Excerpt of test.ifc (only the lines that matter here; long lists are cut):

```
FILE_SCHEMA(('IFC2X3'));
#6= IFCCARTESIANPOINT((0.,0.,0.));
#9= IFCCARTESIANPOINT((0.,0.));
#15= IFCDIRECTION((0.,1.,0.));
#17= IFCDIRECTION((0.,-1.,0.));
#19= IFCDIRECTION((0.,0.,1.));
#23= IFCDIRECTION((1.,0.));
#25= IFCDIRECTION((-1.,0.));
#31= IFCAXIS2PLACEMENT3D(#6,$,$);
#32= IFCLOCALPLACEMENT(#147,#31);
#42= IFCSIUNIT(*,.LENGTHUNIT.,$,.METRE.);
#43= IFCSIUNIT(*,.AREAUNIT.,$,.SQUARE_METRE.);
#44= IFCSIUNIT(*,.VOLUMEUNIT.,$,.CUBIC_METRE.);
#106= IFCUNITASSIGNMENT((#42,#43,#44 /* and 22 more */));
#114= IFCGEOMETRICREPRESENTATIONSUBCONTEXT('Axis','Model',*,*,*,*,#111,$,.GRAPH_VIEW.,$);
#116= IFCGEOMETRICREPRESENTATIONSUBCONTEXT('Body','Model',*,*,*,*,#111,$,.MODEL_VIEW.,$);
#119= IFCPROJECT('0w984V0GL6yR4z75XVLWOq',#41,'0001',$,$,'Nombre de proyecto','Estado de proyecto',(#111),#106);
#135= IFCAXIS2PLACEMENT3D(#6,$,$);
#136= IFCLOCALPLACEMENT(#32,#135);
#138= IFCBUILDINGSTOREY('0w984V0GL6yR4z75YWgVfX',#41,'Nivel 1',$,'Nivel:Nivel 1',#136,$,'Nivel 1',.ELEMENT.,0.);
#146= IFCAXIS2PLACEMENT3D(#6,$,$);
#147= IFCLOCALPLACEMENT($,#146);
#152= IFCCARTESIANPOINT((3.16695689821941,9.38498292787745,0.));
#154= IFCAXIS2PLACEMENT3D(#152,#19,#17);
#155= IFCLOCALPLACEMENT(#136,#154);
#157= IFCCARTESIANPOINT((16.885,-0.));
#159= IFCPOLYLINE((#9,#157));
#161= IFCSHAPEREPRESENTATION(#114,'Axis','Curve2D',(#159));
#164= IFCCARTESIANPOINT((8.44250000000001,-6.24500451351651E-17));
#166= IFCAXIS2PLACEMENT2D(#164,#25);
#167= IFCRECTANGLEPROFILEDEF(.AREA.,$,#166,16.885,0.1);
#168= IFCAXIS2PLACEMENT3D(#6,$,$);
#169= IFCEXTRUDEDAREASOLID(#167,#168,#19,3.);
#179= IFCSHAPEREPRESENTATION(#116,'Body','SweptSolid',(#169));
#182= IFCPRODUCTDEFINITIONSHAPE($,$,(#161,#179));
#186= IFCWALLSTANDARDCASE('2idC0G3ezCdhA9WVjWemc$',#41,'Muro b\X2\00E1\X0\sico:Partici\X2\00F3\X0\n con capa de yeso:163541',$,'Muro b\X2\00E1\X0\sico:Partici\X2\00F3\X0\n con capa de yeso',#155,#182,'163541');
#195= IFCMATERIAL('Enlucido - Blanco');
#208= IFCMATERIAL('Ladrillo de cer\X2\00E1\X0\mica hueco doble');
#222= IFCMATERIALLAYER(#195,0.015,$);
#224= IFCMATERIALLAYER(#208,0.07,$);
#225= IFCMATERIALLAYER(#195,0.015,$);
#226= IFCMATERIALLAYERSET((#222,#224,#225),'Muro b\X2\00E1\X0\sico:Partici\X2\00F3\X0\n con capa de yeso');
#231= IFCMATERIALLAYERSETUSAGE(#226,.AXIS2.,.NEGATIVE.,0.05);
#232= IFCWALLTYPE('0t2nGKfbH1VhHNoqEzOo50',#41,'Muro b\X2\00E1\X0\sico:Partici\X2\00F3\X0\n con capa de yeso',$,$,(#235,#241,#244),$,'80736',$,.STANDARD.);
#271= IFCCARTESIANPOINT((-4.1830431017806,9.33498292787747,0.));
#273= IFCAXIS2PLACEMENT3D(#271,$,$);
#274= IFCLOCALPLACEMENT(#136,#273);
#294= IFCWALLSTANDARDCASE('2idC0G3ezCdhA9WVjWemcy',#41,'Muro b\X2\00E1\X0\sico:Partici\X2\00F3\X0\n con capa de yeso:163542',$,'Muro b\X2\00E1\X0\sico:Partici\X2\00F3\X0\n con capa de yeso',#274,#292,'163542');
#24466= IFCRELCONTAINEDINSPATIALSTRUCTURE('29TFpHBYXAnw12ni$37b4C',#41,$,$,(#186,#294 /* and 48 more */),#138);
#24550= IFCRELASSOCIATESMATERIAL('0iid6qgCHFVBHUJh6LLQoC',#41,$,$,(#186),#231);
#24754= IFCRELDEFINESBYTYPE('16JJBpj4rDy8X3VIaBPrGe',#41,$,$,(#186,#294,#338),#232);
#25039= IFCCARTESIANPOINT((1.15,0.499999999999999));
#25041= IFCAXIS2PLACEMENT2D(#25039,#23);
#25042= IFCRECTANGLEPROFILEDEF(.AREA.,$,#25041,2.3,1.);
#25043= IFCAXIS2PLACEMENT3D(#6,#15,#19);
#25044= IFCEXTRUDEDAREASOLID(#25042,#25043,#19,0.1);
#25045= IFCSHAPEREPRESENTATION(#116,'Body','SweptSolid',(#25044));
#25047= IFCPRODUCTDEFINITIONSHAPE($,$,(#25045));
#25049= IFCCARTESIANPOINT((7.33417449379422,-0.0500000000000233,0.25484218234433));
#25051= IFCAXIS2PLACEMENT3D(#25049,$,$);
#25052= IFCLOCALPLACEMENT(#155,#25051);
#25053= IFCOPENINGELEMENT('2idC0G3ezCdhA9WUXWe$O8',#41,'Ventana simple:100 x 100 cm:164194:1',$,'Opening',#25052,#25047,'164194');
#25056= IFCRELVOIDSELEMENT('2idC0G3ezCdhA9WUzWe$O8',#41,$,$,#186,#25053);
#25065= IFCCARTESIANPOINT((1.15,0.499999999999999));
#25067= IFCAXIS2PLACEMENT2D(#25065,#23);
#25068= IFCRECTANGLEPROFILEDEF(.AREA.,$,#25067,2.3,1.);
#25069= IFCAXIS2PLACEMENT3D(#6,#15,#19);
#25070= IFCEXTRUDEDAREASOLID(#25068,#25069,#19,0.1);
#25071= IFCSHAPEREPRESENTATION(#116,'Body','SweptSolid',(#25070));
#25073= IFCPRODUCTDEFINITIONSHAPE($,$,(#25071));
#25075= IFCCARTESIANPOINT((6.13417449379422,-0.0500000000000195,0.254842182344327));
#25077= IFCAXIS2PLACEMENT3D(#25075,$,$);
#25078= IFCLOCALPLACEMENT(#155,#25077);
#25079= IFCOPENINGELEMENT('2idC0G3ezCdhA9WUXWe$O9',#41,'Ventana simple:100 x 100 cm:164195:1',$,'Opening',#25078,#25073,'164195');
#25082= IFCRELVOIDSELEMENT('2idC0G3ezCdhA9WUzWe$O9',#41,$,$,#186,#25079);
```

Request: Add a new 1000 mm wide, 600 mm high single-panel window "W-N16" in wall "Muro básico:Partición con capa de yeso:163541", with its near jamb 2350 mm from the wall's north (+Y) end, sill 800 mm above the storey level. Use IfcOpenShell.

```python
import numpy as np
import ifcopenshell
import ifcopenshell.api.feature
import ifcopenshell.api.geometry
import ifcopenshell.api.root
import ifcopenshell.api.spatial
import ifcopenshell.api.type
import ifcopenshell.geom
import ifcopenshell.util.element
import ifcopenshell.util.placement
import ifcopenshell.util.representation
import ifcopenshell.util.shape
import ifcopenshell.util.unit

model = ifcopenshell.open("test.ifc")
unit_scale = ifcopenshell.util.unit.calculate_unit_scale(model)
settings = ifcopenshell.geom.settings()


def volume(element):
    """Net volume in cubic metres, openings subtracted."""
    shape = ifcopenshell.geom.create_shape(settings, element)
    return ifcopenshell.util.shape.get_volume(shape.geometry)


wall = model.by_guid("2idC0G3ezCdhA9WVjWemc$")
storey = ifcopenshell.util.element.get_container(wall, ifc_class="IfcBuildingStorey")
context = ifcopenshell.util.representation.get_context(model, "Model", "Body", "MODEL_VIEW")
before = volume(wall)

width, height, from_end, sill = 1, 0.6, 2.35, 0.8  # metres

# The wall runs along its own X axis, and the end named is its -X end.
wall_shape = ifcopenshell.geom.create_shape(settings, wall)
x, y, z = ifcopenshell.util.shape.get_vertices(wall_shape.geometry).T
start = x.min() + from_end
face, thickness = float(y.min()), float(y.max() - y.min())
wall_matrix = ifcopenshell.util.placement.get_local_placement(wall.ObjectPlacement)
level = ifcopenshell.util.placement.get_local_placement(storey.ObjectPlacement)[2, 3]


def in_wall(x, y):
    """Placement at x, y metres in the wall's axes, at sill height."""
    matrix = wall_matrix.copy()
    matrix[:, 3] = wall_matrix @ np.array([x / unit_scale, y / unit_scale, 0.0, 1.0])
    matrix[2, 3] = level + sill / unit_scale
    return matrix


# Opening: a box that overshoots both wall faces by 50 mm.
opening = ifcopenshell.api.root.create_entity(model, ifc_class="IfcOpeningElement")
box = ifcopenshell.api.geometry.add_wall_representation(
    model, context=context, length=width, height=height, thickness=thickness + 0.1
)
ifcopenshell.api.geometry.assign_representation(model, product=opening, representation=box)
ifcopenshell.api.geometry.edit_object_placement(model, product=opening, matrix=in_wall(start, face - 0.05), is_si=False)
ifcopenshell.api.feature.add_feature(model, feature=opening, element=wall)

window = ifcopenshell.api.root.create_entity(model, ifc_class="IfcWindow", name="W-N16")
window.OverallWidth, window.OverallHeight = width / unit_scale, height / unit_scale
body = ifcopenshell.api.geometry.add_window_representation(
    model,
    context=context,
    overall_width=window.OverallWidth,
    overall_height=window.OverallHeight,
    partition_type="SINGLE_PANEL",
)
ifcopenshell.api.geometry.assign_representation(model, product=window, representation=body)
ifcopenshell.api.spatial.assign_container(model, products=[window], relating_structure=storey)
fills = ifcopenshell.api.feature.add_filling(model, opening=opening, element=window)
fills.OwnerHistory = window.OwnerHistory  # required in IFC2X3

# IFC2X3 keeps the operation on the window style.
style = ifcopenshell.api.root.create_entity(model, ifc_class="IfcWindowStyle", name="W-N16")
style.OperationType, style.ConstructionType = "SINGLE_PANEL", "NOTDEFINED"
style.ParameterTakesPrecedence = style.Sizeable = False
ifcopenshell.api.type.assign_type(model, related_objects=[window], relating_type=style)

# Centre the window in the wall's thickness.
ifcopenshell.api.geometry.edit_object_placement(model, product=window, matrix=in_wall(start, face), is_si=False)
window_shape = ifcopenshell.geom.create_shape(settings, window)
depth = ifcopenshell.util.shape.get_vertices(window_shape.geometry)[:, 1]
offset = face + thickness / 2 - (depth.min() + depth.max()) / 2
ifcopenshell.api.geometry.edit_object_placement(model, product=window, matrix=in_wall(start, offset), is_si=False)

after = volume(wall)

print(f"wall volume {before:.3f} -> {after:.3f} m3")

model.write("test_v2.ifc")
```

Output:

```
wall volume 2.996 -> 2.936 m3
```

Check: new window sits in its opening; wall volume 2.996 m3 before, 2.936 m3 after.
